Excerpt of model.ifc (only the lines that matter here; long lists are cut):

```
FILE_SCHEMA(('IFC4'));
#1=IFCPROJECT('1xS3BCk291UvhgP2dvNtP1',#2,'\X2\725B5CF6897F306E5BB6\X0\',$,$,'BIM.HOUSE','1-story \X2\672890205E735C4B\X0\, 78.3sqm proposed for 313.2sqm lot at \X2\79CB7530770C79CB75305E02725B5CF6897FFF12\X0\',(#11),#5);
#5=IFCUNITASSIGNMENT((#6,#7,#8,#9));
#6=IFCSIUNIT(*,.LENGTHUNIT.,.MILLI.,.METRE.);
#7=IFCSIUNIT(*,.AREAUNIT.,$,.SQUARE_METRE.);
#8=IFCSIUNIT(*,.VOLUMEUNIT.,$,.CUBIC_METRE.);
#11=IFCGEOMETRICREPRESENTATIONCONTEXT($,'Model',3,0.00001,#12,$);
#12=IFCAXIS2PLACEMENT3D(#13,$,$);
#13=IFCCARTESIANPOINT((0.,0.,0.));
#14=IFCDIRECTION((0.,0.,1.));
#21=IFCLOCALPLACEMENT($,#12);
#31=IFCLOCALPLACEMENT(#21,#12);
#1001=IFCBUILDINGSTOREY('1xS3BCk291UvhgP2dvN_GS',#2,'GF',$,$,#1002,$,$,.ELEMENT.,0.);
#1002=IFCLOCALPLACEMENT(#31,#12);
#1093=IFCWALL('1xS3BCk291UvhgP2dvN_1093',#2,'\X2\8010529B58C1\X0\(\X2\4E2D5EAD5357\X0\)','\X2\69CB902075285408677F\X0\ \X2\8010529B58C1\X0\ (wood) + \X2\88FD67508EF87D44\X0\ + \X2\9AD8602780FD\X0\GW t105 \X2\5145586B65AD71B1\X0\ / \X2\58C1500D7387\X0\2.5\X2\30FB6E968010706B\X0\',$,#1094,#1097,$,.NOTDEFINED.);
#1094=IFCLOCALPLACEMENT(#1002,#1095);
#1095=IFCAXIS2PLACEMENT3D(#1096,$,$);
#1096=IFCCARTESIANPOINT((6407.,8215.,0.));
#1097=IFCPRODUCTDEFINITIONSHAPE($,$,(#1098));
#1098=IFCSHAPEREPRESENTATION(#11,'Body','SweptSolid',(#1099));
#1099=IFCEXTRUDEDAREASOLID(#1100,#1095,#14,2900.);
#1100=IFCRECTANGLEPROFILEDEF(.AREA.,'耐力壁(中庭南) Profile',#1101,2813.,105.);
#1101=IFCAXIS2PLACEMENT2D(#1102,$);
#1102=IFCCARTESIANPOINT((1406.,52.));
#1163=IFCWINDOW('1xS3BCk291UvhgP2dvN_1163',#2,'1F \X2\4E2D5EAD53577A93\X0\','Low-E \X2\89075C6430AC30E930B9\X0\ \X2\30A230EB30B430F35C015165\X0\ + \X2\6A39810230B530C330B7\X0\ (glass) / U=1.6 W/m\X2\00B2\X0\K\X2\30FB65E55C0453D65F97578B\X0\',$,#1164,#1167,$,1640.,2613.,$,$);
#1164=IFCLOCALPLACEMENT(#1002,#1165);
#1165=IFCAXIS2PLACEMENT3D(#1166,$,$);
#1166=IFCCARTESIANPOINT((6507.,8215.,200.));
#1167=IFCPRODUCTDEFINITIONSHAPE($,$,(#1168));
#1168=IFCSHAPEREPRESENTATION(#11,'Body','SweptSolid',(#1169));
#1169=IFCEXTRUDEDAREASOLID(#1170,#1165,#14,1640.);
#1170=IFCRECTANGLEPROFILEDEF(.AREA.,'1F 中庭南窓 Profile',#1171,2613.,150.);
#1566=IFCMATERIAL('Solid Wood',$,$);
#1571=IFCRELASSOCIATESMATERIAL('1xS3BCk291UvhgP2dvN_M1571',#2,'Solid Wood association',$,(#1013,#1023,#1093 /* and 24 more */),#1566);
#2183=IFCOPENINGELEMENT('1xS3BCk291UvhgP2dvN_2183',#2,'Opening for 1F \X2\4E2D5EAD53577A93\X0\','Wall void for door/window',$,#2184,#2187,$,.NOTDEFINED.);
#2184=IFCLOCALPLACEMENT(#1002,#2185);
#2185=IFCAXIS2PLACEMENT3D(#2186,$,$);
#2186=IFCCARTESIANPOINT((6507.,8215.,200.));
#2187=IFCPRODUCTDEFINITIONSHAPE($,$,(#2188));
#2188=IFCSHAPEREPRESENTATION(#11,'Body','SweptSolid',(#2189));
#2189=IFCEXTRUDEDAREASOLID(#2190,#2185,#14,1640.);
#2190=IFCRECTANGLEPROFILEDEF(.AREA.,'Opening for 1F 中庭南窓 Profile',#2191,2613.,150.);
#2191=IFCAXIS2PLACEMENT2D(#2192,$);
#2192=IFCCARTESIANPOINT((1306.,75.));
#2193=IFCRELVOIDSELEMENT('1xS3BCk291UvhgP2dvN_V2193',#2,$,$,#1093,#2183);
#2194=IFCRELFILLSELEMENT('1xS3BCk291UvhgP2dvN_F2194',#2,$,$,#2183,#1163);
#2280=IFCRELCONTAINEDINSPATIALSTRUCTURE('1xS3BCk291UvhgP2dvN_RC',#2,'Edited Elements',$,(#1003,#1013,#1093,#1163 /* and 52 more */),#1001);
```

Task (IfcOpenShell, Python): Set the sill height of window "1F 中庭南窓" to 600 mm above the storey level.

```python
import numpy as np
import ifcopenshell
import ifcopenshell.api.geometry
import ifcopenshell.geom
import ifcopenshell.util.element
import ifcopenshell.util.placement
import ifcopenshell.util.shape
import ifcopenshell.util.unit

model = ifcopenshell.open("model.ifc")
unit_scale = ifcopenshell.util.unit.calculate_unit_scale(model)

window = model.by_guid("1xS3BCk291UvhgP2dvN_1163")
opening = window.FillsVoids[0].RelatingOpeningElement
storey = ifcopenshell.util.element.get_container(window, ifc_class="IfcBuildingStorey")
level = ifcopenshell.util.placement.get_local_placement(storey.ObjectPlacement)[2, 3]

# The opening's origin need not be at the sill, so measure its lowest point.
shape = ifcopenshell.geom.create_shape(ifcopenshell.geom.settings(), opening)
bottom = ifcopenshell.util.shape.get_shape_bottom_elevation(shape, shape.geometry) / unit_scale
dz = level + 600.0 - bottom

shift = np.array([0.0, 0.0, dz])
# The window is not placed relative to its opening, so move both.
for product in (opening, window):
    matrix = ifcopenshell.util.placement.get_local_placement(product.ObjectPlacement)
    matrix[:3, 3] += shift
    ifcopenshell.api.geometry.edit_object_placement(model, product=product, matrix=matrix, is_si=False)

print(f"moved by {dz * unit_scale:+.3f} m")

model.write("model_v2.ifc")
```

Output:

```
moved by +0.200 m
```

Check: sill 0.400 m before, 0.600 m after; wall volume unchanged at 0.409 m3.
